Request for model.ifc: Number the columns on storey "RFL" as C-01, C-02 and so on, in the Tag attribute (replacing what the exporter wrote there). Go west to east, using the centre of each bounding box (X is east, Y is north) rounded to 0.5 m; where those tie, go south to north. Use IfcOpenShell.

First a look at what the model holds.

```python
import ifcopenshell
import ifcopenshell.util.element
import ifcopenshell.util.placement

model = ifcopenshell.open("model.ifc")
print(model.schema)
storey = next(s for s in model.by_type("IfcBuildingStorey") if s.Name == "RFL")
columns = [e for e in ifcopenshell.util.element.get_decomposition(storey) if e.is_a("IfcColumn")]
for e in sorted(columns, key=lambda e: e.id()):
    origin = ifcopenshell.util.placement.get_local_placement(e.ObjectPlacement)[:3, 3]
    print(e.id(), e.Tag, e.Name, origin.round(2) + 0.0, sep=" | ")
```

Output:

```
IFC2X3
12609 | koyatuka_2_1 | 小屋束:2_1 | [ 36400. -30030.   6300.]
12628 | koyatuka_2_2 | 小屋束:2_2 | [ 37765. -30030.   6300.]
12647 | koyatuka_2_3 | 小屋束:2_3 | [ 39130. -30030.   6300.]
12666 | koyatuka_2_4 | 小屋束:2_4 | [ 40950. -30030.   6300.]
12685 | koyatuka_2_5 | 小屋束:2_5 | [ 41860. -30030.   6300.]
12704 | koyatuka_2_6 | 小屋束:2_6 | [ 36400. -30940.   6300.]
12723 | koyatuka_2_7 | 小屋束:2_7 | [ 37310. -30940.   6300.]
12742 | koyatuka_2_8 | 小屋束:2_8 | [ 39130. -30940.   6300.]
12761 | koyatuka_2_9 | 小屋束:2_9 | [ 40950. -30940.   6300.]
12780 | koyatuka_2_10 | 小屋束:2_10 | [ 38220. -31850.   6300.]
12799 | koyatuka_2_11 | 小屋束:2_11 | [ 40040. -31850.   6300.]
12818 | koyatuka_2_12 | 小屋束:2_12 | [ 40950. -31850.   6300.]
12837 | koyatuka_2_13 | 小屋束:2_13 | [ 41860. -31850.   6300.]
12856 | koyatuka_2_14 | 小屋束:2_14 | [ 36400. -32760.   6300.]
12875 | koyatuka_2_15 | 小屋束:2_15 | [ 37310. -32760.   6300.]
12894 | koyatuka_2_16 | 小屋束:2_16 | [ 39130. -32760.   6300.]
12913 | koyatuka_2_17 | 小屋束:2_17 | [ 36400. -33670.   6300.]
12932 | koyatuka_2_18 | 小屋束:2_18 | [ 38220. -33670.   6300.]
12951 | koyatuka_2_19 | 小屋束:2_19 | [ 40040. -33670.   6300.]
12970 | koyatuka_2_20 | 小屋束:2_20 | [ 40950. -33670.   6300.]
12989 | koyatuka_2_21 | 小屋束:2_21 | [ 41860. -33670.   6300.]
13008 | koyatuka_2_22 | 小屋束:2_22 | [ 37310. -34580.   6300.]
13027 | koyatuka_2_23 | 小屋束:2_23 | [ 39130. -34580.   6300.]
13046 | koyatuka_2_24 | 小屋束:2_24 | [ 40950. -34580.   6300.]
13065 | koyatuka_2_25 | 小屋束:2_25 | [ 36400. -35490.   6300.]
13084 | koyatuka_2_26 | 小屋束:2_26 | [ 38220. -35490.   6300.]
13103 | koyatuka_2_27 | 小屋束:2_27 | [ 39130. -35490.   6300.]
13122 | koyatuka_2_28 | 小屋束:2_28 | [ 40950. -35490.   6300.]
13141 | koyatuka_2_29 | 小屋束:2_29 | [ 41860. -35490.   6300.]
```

```python
import ifcopenshell
import ifcopenshell.geom
import ifcopenshell.util.element
import ifcopenshell.util.shape

model = ifcopenshell.open("model.ifc")
settings = ifcopenshell.geom.settings()
settings.set("use-world-coords", True)


def centre(element):
    shape = ifcopenshell.geom.create_shape(settings, element)
    return ifcopenshell.util.shape.get_bbox_centroid(shape.geometry)


storey = next(s for s in model.by_type("IfcBuildingStorey") if s.Name == "RFL")
columns = [e for e in ifcopenshell.util.element.get_decomposition(storey) if e.is_a("IfcColumn")]

# Insertion points can sit at a corner or the storey origin, so sort by the geometry (in metres).
centres = {e: centre(e) for e in columns}
columns.sort(key=lambda e: (round(centres[e][0] / 0.5), centres[e][1]))

for i, e in enumerate(columns, start=1):
    number = f"C-{i:02d}"
    e.Tag = number
    print(e.id(), number)

model.write("model_edited.ifc")
```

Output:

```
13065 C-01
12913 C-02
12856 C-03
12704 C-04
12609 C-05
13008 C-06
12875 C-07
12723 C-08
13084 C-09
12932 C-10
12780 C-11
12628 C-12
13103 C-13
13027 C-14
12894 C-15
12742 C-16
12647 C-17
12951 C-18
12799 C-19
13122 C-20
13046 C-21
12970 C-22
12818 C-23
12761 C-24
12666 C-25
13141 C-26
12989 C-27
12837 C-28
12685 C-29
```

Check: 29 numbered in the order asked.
